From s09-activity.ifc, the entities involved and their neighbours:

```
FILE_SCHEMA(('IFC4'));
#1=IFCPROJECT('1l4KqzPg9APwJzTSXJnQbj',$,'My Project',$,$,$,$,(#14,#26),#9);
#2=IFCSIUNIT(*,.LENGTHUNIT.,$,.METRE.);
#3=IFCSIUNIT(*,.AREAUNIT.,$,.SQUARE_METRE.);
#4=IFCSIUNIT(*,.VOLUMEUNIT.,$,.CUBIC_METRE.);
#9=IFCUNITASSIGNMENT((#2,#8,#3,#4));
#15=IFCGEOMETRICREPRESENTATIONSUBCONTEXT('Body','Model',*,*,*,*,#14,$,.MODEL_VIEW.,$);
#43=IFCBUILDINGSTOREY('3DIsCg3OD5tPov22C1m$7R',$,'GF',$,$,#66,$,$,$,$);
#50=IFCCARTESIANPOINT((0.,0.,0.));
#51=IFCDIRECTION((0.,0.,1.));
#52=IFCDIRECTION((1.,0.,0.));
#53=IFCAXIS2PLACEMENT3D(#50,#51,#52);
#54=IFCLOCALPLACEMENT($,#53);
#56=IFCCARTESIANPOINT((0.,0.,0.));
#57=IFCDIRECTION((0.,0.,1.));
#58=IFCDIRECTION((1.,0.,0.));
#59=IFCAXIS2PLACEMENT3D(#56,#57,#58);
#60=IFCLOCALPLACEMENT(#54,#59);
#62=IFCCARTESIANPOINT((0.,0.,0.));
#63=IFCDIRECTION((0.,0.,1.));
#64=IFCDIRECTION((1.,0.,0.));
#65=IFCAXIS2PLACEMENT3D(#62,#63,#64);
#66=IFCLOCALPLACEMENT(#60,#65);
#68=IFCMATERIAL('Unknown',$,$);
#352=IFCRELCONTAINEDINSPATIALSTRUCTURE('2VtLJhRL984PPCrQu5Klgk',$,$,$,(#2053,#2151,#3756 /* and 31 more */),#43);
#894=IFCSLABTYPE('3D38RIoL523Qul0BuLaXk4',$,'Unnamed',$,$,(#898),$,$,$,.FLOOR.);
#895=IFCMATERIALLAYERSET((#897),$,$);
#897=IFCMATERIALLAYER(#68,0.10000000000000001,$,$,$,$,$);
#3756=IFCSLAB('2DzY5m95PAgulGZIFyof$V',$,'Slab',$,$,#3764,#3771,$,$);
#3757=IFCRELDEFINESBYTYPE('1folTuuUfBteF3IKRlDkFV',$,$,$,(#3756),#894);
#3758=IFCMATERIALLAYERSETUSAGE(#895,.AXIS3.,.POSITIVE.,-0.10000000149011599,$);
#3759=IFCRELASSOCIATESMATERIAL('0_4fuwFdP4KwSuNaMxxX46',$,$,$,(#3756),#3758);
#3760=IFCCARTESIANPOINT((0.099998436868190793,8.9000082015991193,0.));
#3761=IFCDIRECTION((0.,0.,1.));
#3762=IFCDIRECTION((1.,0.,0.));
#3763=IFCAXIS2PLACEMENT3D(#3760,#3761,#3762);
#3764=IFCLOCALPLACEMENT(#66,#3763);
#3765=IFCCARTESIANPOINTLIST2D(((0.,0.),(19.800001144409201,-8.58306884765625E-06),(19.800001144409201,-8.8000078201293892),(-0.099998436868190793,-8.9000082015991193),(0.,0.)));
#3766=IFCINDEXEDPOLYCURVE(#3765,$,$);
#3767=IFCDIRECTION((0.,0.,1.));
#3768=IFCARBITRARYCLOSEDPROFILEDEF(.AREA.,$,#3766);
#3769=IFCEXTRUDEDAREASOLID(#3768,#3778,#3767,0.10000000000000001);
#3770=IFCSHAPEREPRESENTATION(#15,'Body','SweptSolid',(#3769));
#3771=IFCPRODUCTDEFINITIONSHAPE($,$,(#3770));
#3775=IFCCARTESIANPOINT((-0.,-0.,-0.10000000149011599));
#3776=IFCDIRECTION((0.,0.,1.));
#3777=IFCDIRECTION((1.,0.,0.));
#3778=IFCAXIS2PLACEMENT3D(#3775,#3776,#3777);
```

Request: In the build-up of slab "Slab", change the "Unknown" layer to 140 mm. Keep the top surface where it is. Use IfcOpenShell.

```python
import ifcopenshell
import ifcopenshell.util.element
import ifcopenshell.util.representation
import ifcopenshell.util.unit

model = ifcopenshell.open("s09-activity.ifc")
unit_scale = ifcopenshell.util.unit.calculate_unit_scale(model)

layer_set = model.by_id(895)
layer = next(l for l in layer_set.MaterialLayers if l.Material and l.Material.Name == "Unknown")
change = 0.14 / unit_scale - layer.LayerThickness
layer.LayerThickness += change

# Geometry does not follow the layer set by itself.
slabs = [e for e in ifcopenshell.util.element.get_elements_by_material(model, layer_set) if e.is_a("IfcSlab")]
for slab in sorted(slabs, key=lambda e: e.id()):
    body = ifcopenshell.util.representation.get_representation(slab, "Model", "Body")
    solid = body.Items[0]
    old_depth = solid.Depth
    solid.Depth += change
    # Extruded upwards: lower the start of the extrusion so the top stays.
    x, y, z = solid.Position.Location.Coordinates
    solid.Position.Location = model.createIfcCartesianPoint((x, y, z - change))
    print(slab.id(), f"{old_depth:g} -> {solid.Depth:g}")

# The layers are counted up from the underside, which has moved.
for usage in {ifcopenshell.util.element.get_material(slab) for slab in slabs}:
    usage.OffsetFromReferenceLine -= change

model.write("s09-activity_v2.ifc")
```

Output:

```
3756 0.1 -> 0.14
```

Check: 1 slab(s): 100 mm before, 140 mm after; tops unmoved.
